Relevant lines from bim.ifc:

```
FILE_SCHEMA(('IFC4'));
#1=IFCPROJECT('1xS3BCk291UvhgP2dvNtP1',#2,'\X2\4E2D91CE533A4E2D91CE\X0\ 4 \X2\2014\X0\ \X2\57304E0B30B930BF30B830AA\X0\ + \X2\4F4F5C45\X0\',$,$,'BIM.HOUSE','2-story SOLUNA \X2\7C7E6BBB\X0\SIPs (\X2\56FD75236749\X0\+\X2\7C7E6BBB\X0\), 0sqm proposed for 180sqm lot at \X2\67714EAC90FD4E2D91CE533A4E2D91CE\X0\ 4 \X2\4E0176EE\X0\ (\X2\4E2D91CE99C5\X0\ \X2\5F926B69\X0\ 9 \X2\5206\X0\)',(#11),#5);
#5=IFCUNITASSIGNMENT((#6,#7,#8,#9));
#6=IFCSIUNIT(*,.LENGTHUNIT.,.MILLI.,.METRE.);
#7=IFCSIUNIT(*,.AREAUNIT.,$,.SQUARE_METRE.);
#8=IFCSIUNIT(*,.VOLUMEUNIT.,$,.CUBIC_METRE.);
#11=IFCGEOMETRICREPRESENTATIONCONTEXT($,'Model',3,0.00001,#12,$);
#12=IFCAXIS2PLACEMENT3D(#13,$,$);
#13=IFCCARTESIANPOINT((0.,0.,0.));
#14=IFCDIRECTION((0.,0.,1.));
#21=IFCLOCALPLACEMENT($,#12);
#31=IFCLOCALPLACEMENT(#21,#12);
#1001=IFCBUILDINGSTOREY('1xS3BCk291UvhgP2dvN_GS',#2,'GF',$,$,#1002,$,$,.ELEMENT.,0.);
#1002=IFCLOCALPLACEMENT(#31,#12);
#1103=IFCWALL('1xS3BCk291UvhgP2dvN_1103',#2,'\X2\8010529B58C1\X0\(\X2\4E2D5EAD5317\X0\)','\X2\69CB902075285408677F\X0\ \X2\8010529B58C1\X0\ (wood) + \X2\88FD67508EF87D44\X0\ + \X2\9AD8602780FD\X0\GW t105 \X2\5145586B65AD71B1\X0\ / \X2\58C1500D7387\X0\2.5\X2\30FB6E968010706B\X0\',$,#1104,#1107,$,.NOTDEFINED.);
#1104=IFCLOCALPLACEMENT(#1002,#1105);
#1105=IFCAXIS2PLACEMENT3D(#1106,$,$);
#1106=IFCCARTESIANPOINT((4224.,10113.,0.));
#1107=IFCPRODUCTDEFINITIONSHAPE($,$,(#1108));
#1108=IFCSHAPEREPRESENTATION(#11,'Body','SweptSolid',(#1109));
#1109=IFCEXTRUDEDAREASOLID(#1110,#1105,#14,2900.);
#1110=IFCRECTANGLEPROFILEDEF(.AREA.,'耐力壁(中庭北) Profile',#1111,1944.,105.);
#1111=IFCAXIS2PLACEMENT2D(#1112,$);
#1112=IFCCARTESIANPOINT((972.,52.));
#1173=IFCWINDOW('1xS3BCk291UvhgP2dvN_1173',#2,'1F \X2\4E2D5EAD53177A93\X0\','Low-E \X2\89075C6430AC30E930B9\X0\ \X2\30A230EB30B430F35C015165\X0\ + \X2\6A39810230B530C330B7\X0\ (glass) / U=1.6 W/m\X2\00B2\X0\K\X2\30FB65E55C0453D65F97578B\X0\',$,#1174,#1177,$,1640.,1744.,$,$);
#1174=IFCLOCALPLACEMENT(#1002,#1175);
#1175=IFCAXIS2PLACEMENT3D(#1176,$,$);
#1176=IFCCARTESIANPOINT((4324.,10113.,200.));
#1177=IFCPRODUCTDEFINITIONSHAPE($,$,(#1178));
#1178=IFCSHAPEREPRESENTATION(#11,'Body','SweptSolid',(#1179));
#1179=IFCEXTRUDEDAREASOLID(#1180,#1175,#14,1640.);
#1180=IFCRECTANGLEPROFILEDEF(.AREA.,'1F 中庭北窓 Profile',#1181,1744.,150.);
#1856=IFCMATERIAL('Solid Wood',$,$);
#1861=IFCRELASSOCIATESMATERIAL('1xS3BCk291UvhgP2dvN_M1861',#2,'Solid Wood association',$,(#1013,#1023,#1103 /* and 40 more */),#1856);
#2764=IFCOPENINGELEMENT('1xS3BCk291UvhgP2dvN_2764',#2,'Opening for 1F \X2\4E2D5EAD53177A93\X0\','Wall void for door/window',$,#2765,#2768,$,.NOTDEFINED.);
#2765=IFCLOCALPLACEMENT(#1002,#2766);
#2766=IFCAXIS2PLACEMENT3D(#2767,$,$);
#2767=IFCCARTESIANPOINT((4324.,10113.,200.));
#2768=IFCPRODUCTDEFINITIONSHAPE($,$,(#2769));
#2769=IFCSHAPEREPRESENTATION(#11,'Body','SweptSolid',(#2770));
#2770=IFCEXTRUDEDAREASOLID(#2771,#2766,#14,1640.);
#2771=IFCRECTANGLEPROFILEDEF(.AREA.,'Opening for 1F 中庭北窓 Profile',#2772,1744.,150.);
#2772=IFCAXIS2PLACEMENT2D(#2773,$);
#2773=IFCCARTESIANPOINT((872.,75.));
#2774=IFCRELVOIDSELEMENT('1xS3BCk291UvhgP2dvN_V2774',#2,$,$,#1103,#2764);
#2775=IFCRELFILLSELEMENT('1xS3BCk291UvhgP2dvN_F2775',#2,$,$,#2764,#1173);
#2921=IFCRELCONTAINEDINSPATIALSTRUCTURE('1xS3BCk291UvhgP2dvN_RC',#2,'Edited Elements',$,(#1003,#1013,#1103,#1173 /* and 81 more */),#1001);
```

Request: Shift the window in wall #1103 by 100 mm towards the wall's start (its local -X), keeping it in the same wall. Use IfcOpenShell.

```python
import ifcopenshell
import ifcopenshell.api.geometry
import ifcopenshell.util.placement
import ifcopenshell.util.unit

model = ifcopenshell.open("bim.ifc")
unit_scale = ifcopenshell.util.unit.calculate_unit_scale(model)

window = model.by_guid("1xS3BCk291UvhgP2dvN_1173")
opening = window.FillsVoids[0].RelatingOpeningElement
wall = opening.VoidsElements[0].RelatingBuildingElement

wall_matrix = ifcopenshell.util.placement.get_local_placement(wall.ObjectPlacement)
shift = wall_matrix[:3, 0] * -0.1 / unit_scale
before = ifcopenshell.util.placement.get_local_placement(window.ObjectPlacement)[:3, 3].copy()

# The window is not placed relative to its opening, so move both.
for product in (opening, window):
    matrix = ifcopenshell.util.placement.get_local_placement(product.ObjectPlacement)
    matrix[:3, 3] += shift
    ifcopenshell.api.geometry.edit_object_placement(model, product=product, matrix=matrix, is_si=False)

after = ifcopenshell.util.placement.get_local_placement(window.ObjectPlacement)[:3, 3]
print("window moved by", (after - before).round(3) + 0.0)

model.write("bim_updated.ifc")
```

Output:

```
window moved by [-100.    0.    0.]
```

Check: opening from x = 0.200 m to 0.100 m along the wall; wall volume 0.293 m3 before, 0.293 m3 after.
